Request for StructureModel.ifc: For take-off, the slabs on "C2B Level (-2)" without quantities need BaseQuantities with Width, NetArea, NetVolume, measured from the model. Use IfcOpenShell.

First a look at what the model holds.

```python
import ifcopenshell
import ifcopenshell.util.element
import ifcopenshell.util.unit

model = ifcopenshell.open("StructureModel.ifc")
print(model.schema)
for unit_type in ("LENGTHUNIT", "AREAUNIT", "VOLUMEUNIT"):
    print(unit_type, ifcopenshell.util.unit.calculate_unit_scale(model, unit_type))
storey = next(s for s in model.by_type("IfcBuildingStorey") if s.Name == "C2B Level (-2)")
slabs = [e for e in ifcopenshell.util.element.get_decomposition(storey) if e.is_a("IfcSlab")]
for e in sorted(slabs, key=lambda e: e.id()):
    print(e.id(), e.is_a(), e.Name, list(ifcopenshell.util.element.get_psets(e, qtos_only=True)), sep=" | ")
```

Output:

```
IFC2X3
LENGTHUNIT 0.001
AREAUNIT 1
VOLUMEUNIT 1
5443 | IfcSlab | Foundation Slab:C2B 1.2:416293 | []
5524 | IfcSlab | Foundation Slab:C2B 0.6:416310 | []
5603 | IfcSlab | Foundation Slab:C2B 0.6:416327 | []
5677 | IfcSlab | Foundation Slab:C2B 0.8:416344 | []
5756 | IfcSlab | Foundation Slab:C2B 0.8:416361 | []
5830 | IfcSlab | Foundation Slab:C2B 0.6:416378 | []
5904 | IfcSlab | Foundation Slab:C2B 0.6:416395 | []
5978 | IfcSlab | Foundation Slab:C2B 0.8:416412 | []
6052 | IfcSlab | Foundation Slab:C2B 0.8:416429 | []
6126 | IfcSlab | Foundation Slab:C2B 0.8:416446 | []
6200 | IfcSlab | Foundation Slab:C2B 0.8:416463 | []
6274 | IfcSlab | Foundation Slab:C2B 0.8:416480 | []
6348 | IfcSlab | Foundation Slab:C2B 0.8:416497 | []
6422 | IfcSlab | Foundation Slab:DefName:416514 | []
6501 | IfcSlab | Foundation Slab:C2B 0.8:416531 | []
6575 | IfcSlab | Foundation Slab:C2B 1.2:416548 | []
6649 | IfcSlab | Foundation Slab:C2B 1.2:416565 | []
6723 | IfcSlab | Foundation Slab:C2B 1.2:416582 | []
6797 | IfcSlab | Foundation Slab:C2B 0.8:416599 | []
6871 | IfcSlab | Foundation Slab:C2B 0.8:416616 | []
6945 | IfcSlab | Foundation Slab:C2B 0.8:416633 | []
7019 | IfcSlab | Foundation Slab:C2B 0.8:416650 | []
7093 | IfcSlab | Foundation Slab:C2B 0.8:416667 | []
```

```python
import ifcopenshell
import ifcopenshell.api.pset
import ifcopenshell.geom
import ifcopenshell.util.element
import ifcopenshell.util.shape
import ifcopenshell.util.unit

model = ifcopenshell.open("StructureModel.ifc")
unit_scale = ifcopenshell.util.unit.calculate_unit_scale(model)
area_scale = ifcopenshell.util.unit.calculate_unit_scale(model, "AREAUNIT")
volume_scale = ifcopenshell.util.unit.calculate_unit_scale(model, "VOLUMEUNIT")
settings = ifcopenshell.geom.settings()

storey = next(s for s in model.by_type("IfcBuildingStorey") if s.Name == "C2B Level (-2)")
slabs = [e for e in ifcopenshell.util.element.get_decomposition(storey) if e.is_a("IfcSlab")]

for e in sorted(slabs, key=lambda e: e.id()):
    if ifcopenshell.util.element.get_psets(e, qtos_only=True, should_inherit=False):
        continue
    # Geometry comes back in metres, in the element's own axes.
    shape = ifcopenshell.geom.create_shape(settings, e)
    values = {
        "Width": ifcopenshell.util.shape.get_z(shape.geometry) / unit_scale,
        "NetArea": ifcopenshell.util.shape.get_footprint_area(shape.geometry) / area_scale,
        "NetVolume": ifcopenshell.util.shape.get_volume(shape.geometry) / volume_scale,
    }
    qto = ifcopenshell.api.pset.add_qto(model, product=e, name="BaseQuantities")
    ifcopenshell.api.pset.edit_qto(model, qto=qto, properties=values)
    print(e.id(), {k: round(v, 3) for k, v in values.items()})

model.write("StructureModel-out.ifc")
```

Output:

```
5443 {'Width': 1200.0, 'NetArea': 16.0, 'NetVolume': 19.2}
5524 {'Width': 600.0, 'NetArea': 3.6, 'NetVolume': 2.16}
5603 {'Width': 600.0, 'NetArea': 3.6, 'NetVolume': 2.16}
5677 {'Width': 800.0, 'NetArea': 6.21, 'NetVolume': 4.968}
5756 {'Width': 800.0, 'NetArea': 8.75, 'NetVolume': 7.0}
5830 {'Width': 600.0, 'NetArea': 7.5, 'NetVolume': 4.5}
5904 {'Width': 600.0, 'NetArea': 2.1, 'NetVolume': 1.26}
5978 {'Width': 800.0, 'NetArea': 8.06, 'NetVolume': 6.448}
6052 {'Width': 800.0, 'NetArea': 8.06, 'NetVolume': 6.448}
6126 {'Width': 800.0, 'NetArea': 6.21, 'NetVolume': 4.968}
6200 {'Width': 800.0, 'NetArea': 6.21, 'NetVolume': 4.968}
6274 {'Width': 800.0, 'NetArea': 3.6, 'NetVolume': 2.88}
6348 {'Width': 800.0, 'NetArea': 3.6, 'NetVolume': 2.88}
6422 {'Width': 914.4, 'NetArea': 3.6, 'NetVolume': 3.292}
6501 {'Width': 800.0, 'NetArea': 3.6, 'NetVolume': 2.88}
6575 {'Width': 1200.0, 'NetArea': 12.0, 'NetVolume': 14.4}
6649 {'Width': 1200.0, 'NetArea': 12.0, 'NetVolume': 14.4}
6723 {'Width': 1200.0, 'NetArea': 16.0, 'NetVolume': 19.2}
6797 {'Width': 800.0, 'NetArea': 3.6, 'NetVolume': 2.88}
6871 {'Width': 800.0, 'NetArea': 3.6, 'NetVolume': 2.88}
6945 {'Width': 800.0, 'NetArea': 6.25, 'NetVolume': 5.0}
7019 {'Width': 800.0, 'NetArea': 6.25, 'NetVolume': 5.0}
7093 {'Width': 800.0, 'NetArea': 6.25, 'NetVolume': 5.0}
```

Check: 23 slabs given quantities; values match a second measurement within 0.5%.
